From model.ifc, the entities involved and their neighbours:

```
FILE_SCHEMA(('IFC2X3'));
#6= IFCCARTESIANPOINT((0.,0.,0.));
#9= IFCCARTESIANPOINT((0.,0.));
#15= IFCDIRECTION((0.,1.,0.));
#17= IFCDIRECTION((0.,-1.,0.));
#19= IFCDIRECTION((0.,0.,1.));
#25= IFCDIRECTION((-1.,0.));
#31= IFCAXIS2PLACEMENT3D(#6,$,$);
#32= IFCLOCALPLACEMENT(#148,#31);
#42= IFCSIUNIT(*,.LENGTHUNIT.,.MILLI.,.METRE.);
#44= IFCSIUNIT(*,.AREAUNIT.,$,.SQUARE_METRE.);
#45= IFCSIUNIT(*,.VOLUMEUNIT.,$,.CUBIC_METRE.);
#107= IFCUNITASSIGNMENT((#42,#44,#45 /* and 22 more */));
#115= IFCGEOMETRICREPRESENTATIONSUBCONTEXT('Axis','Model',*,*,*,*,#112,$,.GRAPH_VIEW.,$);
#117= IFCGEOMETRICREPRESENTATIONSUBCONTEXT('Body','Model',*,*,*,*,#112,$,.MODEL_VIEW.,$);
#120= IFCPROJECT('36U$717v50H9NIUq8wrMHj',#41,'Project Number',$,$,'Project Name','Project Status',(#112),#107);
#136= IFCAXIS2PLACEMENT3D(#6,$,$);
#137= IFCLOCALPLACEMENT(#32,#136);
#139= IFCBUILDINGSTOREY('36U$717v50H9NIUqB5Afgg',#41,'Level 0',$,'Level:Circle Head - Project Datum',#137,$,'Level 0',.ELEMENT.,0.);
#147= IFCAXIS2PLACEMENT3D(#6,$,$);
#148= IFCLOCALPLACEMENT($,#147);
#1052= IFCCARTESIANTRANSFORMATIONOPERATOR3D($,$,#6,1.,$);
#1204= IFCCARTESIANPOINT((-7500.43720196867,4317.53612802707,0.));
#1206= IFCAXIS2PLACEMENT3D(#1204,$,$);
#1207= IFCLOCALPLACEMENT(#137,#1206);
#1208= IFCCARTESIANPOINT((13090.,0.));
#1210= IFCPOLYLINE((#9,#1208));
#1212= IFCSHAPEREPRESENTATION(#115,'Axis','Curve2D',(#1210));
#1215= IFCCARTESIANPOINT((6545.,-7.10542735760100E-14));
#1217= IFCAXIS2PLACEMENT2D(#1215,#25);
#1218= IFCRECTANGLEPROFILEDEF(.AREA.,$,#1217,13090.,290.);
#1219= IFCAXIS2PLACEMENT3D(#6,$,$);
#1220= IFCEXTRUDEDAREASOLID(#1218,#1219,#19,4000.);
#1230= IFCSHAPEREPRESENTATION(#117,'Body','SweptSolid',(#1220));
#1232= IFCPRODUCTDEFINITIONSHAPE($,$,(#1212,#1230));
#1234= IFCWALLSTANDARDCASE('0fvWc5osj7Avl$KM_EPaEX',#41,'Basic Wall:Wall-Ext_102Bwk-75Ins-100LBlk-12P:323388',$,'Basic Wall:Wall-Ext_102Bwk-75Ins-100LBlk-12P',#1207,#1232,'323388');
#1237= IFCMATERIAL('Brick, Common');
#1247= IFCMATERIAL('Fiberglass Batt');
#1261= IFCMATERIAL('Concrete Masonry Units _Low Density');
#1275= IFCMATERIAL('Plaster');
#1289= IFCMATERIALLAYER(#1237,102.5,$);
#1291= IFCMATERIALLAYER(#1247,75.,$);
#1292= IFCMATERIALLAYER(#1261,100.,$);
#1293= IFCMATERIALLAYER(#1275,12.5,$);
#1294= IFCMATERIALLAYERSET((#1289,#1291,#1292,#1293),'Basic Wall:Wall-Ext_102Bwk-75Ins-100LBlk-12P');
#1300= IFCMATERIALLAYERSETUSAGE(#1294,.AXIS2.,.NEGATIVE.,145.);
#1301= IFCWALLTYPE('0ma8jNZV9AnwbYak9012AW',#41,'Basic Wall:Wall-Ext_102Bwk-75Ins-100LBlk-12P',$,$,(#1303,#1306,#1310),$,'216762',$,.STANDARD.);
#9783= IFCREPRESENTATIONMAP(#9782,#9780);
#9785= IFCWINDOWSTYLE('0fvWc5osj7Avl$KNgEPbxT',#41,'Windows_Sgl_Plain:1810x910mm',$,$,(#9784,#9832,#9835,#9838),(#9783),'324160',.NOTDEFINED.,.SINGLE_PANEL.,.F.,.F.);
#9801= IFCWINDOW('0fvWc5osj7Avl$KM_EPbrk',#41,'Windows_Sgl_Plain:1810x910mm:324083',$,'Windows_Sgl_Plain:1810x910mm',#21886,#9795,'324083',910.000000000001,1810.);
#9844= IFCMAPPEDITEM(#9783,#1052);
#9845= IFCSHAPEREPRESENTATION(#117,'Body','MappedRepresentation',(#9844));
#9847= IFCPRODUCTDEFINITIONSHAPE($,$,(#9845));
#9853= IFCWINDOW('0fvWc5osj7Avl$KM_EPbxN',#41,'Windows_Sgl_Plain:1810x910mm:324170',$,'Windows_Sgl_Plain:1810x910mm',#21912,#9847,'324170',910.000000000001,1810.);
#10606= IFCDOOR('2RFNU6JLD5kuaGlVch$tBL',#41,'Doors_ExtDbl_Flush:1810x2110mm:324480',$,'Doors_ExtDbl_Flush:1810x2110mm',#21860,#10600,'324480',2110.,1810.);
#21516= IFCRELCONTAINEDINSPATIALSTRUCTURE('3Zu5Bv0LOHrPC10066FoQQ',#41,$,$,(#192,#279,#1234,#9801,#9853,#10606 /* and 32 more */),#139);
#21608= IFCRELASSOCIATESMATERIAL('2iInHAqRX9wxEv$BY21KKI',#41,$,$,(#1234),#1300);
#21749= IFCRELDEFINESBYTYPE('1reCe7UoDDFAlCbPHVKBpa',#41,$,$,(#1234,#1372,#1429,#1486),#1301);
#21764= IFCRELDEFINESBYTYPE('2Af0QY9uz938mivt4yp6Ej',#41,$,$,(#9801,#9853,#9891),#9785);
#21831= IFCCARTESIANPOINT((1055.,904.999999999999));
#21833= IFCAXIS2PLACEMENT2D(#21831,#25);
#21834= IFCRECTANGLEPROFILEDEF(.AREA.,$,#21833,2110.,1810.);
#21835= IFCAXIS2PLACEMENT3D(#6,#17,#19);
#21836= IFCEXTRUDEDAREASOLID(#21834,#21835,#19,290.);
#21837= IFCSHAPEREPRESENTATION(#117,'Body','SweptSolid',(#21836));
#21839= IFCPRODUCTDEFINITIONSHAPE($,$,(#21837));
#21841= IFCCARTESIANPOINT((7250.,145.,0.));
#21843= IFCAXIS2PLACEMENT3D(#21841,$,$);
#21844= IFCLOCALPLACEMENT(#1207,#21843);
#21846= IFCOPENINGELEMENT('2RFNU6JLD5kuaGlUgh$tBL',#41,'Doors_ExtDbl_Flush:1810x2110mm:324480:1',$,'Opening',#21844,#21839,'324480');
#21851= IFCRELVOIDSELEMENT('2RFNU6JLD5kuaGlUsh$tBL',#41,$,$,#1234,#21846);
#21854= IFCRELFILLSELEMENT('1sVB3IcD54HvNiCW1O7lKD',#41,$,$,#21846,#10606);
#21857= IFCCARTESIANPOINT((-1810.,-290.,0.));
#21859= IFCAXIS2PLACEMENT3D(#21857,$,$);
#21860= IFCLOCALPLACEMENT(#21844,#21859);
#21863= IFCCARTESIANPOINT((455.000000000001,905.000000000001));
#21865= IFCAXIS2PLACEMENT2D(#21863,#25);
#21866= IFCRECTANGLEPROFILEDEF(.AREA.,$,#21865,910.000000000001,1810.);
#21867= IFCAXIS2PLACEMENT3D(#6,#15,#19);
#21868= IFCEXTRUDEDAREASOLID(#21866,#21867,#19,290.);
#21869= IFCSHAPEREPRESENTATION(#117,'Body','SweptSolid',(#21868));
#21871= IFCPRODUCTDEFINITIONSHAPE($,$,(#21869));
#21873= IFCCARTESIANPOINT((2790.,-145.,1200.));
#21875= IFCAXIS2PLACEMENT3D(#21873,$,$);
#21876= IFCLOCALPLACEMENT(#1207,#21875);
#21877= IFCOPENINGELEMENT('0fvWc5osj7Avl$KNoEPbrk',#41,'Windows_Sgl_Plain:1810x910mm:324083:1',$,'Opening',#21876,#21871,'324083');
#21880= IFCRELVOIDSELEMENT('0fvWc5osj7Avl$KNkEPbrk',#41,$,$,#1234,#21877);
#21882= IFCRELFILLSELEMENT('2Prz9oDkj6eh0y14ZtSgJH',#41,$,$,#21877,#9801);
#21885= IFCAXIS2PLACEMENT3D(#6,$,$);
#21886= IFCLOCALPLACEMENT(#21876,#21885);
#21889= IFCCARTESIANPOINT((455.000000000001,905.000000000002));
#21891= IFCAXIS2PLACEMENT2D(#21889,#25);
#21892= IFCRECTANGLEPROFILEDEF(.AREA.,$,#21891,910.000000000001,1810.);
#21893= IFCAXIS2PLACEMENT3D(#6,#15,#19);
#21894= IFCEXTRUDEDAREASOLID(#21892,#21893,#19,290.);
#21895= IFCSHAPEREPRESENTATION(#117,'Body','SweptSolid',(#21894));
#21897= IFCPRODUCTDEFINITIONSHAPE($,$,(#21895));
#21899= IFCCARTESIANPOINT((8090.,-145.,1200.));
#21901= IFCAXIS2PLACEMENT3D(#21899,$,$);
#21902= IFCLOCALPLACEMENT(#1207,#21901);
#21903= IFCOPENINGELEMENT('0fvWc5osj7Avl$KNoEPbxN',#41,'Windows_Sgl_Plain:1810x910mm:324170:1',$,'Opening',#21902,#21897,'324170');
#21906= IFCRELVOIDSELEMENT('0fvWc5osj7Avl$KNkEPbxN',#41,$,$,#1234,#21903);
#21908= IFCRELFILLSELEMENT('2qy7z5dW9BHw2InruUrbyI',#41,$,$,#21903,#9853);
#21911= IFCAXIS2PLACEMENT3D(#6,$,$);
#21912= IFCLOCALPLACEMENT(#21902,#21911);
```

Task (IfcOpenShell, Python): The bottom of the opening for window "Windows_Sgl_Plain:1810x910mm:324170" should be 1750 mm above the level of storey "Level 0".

```python
import numpy as np
import ifcopenshell
import ifcopenshell.api.geometry
import ifcopenshell.geom
import ifcopenshell.util.element
import ifcopenshell.util.placement
import ifcopenshell.util.shape
import ifcopenshell.util.unit

model = ifcopenshell.open("model.ifc")
unit_scale = ifcopenshell.util.unit.calculate_unit_scale(model)

window = model.by_guid("0fvWc5osj7Avl$KM_EPbxN")
opening = window.FillsVoids[0].RelatingOpeningElement
storey = ifcopenshell.util.element.get_container(window, ifc_class="IfcBuildingStorey")
level = ifcopenshell.util.placement.get_local_placement(storey.ObjectPlacement)[2, 3]

# The opening's origin need not be at the sill, so measure its lowest point.
shape = ifcopenshell.geom.create_shape(ifcopenshell.geom.settings(), opening)
bottom = ifcopenshell.util.shape.get_shape_bottom_elevation(shape, shape.geometry) / unit_scale
dz = level + 1.75 / unit_scale - bottom

shift = np.array([0.0, 0.0, dz])
# The window is placed relative to its opening, so it follows when the opening moves.
matrix = ifcopenshell.util.placement.get_local_placement(opening.ObjectPlacement)
matrix[:3, 3] += shift
ifcopenshell.api.geometry.edit_object_placement(
    model, product=opening, matrix=matrix, is_si=False, should_transform_children=True
)

print(f"moved by {dz * unit_scale:+.3f} m")

model.write("model_updated.ifc")
```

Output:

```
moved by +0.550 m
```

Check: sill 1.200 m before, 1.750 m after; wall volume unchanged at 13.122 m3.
